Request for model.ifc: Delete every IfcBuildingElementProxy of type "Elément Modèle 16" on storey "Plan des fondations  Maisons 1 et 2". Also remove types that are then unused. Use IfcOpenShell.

First a look at what the model holds.

```python
import ifcopenshell
import ifcopenshell.util.element

model = ifcopenshell.open("model.ifc")
print(model.schema)
storey = next(s for s in model.by_type("IfcBuildingStorey") if s.Name == "Plan des fondations  Maisons 1 et 2")
proxies = [e for e in ifcopenshell.util.element.get_decomposition(storey) if e.is_a("IfcBuildingElementProxy")]
seen = {}
for e in proxies:
    element_type = ifcopenshell.util.element.get_type(e)
    name = element_type.Name if element_type not in (None, e) else None
    seen[name] = seen.get(name, 0) + 1
for name, count in sorted(seen.items(), key=str):
    print(count, "x", name)
```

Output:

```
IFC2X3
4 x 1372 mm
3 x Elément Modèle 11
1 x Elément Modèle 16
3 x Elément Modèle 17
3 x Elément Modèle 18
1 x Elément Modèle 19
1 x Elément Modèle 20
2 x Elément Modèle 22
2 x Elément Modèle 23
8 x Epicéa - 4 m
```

```python
import ifcopenshell
import ifcopenshell.api.root
import ifcopenshell.util.element

model = ifcopenshell.open("model.ifc")

storey = next(s for s in model.by_type("IfcBuildingStorey") if s.Name == "Plan des fondations  Maisons 1 et 2")
proxies = [e for e in ifcopenshell.util.element.get_decomposition(storey) if e.is_a("IfcBuildingElementProxy")]
targets = [e for e in proxies if (t := ifcopenshell.util.element.get_type(e)) not in (None, e) and t.Name == "Elément Modèle 16"]
types = {ifcopenshell.util.element.get_type(e) for e in targets} - {None, *targets}

for e in targets:
    ifcopenshell.api.root.remove_product(model, product=e)
print(len(targets), "removed")

unused = [t for t in types if not ifcopenshell.util.element.get_types(t)]
for t in unused:
    ifcopenshell.api.root.remove_product(model, product=t)
print(len(unused), "unused types removed")

model.write("model_rev.ifc")
```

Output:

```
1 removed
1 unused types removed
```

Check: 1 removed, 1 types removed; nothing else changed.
